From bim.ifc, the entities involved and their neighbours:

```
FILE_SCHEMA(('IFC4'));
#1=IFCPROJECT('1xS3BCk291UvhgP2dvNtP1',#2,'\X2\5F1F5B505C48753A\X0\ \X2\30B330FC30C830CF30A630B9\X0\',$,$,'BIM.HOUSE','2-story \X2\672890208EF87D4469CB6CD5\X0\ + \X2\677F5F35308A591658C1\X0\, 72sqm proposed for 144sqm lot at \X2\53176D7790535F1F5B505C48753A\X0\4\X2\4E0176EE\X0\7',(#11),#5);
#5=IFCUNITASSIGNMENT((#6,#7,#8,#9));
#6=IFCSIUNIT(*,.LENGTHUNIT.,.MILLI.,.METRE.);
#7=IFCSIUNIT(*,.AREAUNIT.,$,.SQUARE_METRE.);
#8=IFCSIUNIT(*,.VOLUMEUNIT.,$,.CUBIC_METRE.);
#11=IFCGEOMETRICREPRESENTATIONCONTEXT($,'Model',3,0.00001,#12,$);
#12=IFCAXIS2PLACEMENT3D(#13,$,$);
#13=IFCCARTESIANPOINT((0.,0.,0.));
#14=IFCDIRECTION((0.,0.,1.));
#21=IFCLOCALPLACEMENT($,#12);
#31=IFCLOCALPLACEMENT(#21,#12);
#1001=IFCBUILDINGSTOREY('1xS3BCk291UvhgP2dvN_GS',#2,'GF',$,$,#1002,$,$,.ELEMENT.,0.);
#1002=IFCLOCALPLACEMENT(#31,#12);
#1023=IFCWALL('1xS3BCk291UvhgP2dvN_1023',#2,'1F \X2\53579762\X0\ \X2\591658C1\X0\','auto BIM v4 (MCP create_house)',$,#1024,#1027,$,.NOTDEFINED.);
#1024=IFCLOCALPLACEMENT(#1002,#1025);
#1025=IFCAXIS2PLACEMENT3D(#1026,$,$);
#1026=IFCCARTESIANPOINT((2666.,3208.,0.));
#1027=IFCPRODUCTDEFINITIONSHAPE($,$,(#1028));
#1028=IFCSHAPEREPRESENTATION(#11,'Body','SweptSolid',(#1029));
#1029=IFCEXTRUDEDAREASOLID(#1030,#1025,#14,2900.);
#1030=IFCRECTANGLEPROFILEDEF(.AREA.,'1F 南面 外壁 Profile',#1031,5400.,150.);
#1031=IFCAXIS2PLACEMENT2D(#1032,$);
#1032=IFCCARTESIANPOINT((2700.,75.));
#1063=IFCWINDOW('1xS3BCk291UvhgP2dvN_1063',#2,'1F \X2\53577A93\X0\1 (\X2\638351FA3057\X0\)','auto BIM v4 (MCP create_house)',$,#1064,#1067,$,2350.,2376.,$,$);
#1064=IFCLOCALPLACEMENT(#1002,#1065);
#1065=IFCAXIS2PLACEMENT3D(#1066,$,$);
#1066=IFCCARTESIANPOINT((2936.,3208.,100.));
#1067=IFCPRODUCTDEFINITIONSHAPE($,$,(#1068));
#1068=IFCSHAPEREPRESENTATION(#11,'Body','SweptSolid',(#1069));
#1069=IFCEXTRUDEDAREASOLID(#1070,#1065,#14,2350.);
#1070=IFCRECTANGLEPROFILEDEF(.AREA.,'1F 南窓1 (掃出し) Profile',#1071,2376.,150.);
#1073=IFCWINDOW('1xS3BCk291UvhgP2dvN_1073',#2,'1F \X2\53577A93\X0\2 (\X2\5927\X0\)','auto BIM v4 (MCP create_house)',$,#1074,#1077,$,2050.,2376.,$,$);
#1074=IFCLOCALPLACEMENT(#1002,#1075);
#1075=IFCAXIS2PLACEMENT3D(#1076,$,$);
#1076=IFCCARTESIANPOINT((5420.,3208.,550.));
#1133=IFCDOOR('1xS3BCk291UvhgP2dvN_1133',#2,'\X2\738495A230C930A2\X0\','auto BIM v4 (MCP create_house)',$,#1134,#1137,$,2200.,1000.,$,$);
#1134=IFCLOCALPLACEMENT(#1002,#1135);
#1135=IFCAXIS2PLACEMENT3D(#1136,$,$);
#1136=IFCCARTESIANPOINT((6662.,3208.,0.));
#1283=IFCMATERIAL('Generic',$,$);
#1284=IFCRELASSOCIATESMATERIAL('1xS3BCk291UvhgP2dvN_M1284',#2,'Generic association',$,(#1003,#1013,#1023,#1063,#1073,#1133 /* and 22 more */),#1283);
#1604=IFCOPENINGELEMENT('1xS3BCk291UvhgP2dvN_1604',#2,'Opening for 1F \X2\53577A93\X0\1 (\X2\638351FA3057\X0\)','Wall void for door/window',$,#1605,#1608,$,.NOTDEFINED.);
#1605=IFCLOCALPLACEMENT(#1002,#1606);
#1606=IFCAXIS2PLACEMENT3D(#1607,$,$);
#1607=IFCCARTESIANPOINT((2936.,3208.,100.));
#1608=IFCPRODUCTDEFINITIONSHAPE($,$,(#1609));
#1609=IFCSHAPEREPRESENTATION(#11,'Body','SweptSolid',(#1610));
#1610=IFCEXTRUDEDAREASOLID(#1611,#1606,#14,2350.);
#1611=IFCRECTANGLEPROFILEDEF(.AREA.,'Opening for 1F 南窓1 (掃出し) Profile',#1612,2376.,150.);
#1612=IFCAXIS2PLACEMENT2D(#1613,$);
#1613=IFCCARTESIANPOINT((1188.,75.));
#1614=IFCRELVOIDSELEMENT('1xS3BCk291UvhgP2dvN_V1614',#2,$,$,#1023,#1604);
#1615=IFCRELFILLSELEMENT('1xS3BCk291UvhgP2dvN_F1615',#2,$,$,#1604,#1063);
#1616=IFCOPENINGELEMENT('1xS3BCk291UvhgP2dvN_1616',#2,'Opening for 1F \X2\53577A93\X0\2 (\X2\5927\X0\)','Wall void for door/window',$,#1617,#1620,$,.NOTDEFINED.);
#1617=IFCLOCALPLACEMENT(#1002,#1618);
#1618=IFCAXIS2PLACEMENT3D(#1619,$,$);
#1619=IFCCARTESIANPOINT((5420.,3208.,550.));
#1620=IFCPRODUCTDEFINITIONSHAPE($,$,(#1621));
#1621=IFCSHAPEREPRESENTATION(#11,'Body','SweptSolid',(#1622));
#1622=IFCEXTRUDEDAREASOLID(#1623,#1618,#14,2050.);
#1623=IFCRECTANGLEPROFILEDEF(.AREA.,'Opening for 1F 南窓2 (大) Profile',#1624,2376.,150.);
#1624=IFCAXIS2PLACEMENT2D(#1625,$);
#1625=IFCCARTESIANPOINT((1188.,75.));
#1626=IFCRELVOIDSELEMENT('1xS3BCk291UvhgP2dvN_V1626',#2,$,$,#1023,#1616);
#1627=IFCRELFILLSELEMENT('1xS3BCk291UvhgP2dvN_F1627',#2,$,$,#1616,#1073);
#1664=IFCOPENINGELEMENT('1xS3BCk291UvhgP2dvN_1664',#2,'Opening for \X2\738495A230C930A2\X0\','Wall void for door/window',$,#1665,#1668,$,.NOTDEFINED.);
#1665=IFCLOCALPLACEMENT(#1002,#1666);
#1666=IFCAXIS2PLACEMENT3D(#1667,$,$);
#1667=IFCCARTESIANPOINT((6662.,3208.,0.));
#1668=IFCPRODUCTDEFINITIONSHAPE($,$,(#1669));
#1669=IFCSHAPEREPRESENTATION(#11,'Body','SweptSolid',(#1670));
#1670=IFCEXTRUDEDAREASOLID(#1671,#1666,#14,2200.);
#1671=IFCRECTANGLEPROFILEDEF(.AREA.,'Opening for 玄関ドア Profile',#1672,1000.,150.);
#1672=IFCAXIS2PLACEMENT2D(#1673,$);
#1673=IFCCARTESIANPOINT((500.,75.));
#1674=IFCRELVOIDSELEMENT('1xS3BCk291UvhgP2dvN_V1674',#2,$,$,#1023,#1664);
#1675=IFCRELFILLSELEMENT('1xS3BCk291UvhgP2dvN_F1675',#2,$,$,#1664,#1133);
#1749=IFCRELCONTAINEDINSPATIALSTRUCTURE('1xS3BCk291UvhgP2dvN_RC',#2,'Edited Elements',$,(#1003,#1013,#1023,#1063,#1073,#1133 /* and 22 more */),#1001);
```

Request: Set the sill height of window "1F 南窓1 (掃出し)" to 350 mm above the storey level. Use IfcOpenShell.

```python
import numpy as np
import ifcopenshell
import ifcopenshell.api.geometry
import ifcopenshell.geom
import ifcopenshell.util.element
import ifcopenshell.util.placement
import ifcopenshell.util.shape
import ifcopenshell.util.unit

model = ifcopenshell.open("bim.ifc")
unit_scale = ifcopenshell.util.unit.calculate_unit_scale(model)

window = model.by_id(1063)
opening = window.FillsVoids[0].RelatingOpeningElement
storey = ifcopenshell.util.element.get_container(window, ifc_class="IfcBuildingStorey")
level = ifcopenshell.util.placement.get_local_placement(storey.ObjectPlacement)[2, 3]

# The opening's origin need not be at the sill, so measure its lowest point.
shape = ifcopenshell.geom.create_shape(ifcopenshell.geom.settings(), opening)
bottom = ifcopenshell.util.shape.get_shape_bottom_elevation(shape, shape.geometry) / unit_scale
dz = level + 0.35 / unit_scale - bottom

shift = np.array([0.0, 0.0, dz])
# The window is not placed relative to its opening, so move both.
for product in (opening, window):
    matrix = ifcopenshell.util.placement.get_local_placement(product.ObjectPlacement)
    matrix[:3, 3] += shift
    ifcopenshell.api.geometry.edit_object_placement(model, product=product, matrix=matrix, is_si=False)

print(f"moved by {dz * unit_scale:+.3f} m")

model.write("bim_rev.ifc")
```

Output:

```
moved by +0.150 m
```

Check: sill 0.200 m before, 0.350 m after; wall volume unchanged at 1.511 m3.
